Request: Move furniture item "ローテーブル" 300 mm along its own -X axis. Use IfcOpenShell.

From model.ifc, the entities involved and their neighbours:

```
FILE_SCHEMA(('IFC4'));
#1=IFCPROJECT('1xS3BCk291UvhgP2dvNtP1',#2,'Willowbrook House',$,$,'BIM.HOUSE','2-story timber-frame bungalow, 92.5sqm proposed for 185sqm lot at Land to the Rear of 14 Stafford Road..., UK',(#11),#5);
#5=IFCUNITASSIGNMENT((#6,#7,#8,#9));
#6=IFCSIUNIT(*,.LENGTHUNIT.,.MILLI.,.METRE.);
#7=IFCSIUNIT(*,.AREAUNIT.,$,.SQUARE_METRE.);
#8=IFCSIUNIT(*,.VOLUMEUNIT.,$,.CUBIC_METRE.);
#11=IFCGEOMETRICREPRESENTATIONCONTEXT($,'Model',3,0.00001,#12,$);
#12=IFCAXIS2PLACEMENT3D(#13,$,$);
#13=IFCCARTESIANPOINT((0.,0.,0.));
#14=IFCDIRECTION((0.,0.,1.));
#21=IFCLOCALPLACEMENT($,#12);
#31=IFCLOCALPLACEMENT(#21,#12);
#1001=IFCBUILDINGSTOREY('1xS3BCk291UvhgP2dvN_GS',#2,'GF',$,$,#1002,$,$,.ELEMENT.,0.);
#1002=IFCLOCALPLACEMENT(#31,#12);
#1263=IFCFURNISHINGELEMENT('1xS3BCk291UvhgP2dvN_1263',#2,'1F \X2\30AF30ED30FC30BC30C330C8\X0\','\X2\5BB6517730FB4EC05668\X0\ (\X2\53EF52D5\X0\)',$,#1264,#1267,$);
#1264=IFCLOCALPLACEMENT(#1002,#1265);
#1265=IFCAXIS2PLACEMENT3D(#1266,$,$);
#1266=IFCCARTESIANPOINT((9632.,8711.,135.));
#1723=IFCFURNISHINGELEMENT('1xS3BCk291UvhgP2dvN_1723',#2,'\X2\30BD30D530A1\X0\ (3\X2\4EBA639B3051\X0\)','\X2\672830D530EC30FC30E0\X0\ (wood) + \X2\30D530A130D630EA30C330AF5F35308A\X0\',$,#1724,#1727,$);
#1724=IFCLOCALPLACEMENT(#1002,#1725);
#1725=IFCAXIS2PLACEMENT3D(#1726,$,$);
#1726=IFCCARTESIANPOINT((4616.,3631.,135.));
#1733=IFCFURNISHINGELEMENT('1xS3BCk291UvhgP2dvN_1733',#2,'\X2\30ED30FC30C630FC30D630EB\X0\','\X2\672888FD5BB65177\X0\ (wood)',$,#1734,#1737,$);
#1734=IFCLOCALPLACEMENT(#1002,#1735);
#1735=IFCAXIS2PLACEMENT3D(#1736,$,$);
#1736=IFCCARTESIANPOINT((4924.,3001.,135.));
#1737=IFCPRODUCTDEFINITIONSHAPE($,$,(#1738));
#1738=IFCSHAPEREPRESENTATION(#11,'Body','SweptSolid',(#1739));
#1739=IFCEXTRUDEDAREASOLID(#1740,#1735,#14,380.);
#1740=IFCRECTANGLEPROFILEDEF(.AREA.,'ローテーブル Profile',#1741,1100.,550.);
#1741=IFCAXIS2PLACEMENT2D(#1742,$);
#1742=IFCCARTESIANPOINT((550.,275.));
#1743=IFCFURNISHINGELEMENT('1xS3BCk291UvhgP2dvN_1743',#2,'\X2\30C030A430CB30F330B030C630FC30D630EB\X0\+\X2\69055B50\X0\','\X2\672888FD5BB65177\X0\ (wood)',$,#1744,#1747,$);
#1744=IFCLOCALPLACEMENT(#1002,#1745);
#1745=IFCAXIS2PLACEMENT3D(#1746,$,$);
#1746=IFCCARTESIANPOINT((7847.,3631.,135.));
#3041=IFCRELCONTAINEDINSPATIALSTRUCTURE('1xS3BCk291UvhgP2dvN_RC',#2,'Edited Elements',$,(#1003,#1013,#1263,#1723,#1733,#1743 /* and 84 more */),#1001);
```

```python
import ifcopenshell
import ifcopenshell.api.geometry
import ifcopenshell.util.placement
import ifcopenshell.util.unit

model = ifcopenshell.open("model.ifc")
unit_scale = ifcopenshell.util.unit.calculate_unit_scale(model)

item = model.by_guid("1xS3BCk291UvhgP2dvN_1733")
matrix = ifcopenshell.util.placement.get_local_placement(item.ObjectPlacement)
matrix[:3, 3] -= matrix[:3, 0] * 0.3 / unit_scale
ifcopenshell.api.geometry.edit_object_placement(model, product=item, matrix=matrix, is_si=False)

print(ifcopenshell.util.placement.get_local_placement(item.ObjectPlacement).round(3) + 0.0)

model.write("model-out.ifc")
```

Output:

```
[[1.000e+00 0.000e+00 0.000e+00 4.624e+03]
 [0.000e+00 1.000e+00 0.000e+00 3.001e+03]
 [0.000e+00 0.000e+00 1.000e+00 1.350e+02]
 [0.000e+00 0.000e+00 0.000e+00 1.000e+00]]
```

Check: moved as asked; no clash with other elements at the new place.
